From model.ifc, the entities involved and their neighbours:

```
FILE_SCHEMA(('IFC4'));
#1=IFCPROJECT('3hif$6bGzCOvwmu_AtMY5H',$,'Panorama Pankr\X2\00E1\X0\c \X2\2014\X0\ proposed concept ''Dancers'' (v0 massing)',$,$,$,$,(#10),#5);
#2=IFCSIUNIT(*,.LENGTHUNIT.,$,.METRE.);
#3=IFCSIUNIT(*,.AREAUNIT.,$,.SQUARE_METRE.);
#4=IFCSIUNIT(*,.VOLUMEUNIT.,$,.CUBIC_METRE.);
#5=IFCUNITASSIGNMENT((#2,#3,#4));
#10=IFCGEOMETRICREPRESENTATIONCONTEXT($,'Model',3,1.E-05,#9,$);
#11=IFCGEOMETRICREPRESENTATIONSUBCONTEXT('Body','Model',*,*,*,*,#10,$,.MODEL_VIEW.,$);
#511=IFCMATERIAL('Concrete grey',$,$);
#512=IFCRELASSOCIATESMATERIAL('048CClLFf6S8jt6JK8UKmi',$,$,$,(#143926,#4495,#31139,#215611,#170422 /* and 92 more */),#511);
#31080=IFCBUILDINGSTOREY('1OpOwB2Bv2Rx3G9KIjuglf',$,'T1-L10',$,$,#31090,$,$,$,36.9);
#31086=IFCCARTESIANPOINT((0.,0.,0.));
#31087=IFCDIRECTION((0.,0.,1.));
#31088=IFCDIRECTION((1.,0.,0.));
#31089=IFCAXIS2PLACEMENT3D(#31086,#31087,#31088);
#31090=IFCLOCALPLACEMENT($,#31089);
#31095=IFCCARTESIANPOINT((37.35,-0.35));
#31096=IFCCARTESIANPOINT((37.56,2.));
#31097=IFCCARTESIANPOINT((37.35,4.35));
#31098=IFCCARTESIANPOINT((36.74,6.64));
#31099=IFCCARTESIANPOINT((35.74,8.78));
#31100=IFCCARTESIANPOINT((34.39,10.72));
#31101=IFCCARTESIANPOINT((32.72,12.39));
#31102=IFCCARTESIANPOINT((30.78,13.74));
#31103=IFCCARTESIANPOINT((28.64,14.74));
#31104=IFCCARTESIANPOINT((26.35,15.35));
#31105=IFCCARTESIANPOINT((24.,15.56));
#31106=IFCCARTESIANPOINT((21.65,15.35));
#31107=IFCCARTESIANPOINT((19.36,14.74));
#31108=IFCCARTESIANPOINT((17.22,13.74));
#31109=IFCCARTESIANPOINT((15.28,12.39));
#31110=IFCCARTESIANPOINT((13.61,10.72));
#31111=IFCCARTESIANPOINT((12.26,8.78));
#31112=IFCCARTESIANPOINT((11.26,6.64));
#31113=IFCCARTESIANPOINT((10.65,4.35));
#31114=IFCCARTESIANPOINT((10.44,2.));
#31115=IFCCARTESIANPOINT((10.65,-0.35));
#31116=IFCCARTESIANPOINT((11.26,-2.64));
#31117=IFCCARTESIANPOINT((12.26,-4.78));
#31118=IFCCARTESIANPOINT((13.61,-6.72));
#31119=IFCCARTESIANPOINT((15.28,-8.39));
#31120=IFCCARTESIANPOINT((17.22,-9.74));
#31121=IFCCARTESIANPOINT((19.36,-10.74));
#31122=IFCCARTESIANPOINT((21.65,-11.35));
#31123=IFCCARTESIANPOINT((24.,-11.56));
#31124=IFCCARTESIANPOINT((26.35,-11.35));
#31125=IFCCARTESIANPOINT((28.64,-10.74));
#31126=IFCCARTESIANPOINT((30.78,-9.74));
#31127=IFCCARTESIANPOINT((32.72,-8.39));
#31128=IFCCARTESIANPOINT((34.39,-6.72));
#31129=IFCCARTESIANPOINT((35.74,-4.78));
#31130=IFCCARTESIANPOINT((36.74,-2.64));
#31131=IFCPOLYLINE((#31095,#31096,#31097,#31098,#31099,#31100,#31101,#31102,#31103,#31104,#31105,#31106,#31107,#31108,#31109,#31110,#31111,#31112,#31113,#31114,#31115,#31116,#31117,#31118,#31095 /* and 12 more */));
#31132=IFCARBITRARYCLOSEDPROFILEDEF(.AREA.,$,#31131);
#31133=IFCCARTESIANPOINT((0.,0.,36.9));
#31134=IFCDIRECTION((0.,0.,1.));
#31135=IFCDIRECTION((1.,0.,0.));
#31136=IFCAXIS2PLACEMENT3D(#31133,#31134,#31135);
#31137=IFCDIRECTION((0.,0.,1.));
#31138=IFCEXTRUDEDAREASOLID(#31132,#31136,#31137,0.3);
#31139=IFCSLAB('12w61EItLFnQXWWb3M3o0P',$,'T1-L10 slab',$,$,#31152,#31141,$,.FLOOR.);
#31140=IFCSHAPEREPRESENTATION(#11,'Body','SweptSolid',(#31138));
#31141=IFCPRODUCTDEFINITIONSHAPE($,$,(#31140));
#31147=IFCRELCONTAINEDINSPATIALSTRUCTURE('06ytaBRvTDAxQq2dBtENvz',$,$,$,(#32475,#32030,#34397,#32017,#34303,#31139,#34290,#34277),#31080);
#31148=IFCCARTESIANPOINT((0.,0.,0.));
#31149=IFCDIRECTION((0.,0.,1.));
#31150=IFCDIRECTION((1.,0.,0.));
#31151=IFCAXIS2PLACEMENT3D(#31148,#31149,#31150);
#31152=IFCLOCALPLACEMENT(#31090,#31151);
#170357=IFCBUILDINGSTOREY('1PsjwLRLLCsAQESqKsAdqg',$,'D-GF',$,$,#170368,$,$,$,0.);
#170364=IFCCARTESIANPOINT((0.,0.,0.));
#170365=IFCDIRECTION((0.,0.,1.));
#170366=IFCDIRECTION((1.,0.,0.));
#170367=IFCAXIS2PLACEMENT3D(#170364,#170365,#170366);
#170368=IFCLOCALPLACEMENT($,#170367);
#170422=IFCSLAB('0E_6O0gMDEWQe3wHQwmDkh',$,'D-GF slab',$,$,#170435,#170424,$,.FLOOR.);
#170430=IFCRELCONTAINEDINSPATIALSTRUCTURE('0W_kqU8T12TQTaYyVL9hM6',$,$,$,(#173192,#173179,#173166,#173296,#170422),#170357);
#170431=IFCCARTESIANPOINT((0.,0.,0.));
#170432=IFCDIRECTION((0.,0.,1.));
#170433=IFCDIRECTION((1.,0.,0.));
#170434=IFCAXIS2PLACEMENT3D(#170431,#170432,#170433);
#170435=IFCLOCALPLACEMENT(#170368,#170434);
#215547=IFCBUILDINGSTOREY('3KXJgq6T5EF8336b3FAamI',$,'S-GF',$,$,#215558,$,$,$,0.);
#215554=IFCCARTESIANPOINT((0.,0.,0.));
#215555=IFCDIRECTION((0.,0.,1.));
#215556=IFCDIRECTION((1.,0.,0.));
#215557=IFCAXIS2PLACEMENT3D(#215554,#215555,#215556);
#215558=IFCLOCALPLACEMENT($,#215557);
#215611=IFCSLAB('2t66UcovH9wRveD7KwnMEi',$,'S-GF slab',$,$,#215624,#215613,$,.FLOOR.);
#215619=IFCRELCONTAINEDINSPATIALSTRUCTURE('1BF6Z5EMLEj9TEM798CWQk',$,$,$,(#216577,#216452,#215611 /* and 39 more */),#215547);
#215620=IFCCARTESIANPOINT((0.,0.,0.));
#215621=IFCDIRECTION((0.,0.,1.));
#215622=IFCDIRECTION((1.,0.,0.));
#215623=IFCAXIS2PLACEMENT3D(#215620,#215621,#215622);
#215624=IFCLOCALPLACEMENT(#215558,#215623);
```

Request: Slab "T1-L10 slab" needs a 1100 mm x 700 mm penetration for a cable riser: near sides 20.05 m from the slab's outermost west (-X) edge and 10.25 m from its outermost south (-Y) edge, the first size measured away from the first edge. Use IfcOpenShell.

```python
import numpy as np
import ifcopenshell
import ifcopenshell.api.feature
import ifcopenshell.api.geometry
import ifcopenshell.api.root
import ifcopenshell.geom
import ifcopenshell.util.placement
import ifcopenshell.util.representation
import ifcopenshell.util.shape
import ifcopenshell.util.unit

model = ifcopenshell.open("model.ifc")
unit_scale = ifcopenshell.util.unit.calculate_unit_scale(model)
settings = ifcopenshell.geom.settings()


def volume(element):
    """Net volume in cubic metres, openings subtracted."""
    shape = ifcopenshell.geom.create_shape(settings, element)
    return ifcopenshell.util.shape.get_volume(shape.geometry)


slab = model.by_guid("12w61EItLFnQXWWb3M3o0P")
before = volume(slab)

# Extent in the slab's own axes, in metres. The edges named are its -X and -Y sides.
slab_shape = ifcopenshell.geom.create_shape(settings, slab)
vertices = ifcopenshell.util.shape.get_vertices(slab_shape.geometry)
x_min, y_min, bottom = vertices.min(axis=0)
top = vertices[:, 2].max()

opening = ifcopenshell.api.root.create_entity(model, ifc_class="IfcOpeningElement", name="Cable riser opening", predefined_type="OPENING")
context = ifcopenshell.util.representation.get_context(model, "Model", "Body", "MODEL_VIEW")
width, depth = 1.1, 0.7
outline = [(0.0, 0.0), (width, 0.0), (width, depth), (0.0, depth), (0.0, 0.0)]
# Overshoot both faces by 50 mm so the cut is clean.
shape = ifcopenshell.api.geometry.add_slab_representation(
    model, context=context, depth=top - bottom + 0.1, polyline=outline
)
ifcopenshell.api.geometry.assign_representation(model, product=opening, representation=shape)

matrix = ifcopenshell.util.placement.get_local_placement(slab.ObjectPlacement)
matrix[:, 3] = matrix @ np.append(np.array([x_min + 20.05, y_min + 10.25, bottom - 0.05]) / unit_scale, 1.0)
ifcopenshell.api.geometry.edit_object_placement(model, product=opening, matrix=matrix, is_si=False)
ifcopenshell.api.feature.add_feature(model, feature=opening, element=slab)

after = volume(slab)

print(f"slab volume {before:.3f} -> {after:.3f} m3")

model.write("model_edited.ifc")
```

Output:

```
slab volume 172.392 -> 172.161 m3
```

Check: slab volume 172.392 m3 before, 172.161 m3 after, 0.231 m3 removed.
